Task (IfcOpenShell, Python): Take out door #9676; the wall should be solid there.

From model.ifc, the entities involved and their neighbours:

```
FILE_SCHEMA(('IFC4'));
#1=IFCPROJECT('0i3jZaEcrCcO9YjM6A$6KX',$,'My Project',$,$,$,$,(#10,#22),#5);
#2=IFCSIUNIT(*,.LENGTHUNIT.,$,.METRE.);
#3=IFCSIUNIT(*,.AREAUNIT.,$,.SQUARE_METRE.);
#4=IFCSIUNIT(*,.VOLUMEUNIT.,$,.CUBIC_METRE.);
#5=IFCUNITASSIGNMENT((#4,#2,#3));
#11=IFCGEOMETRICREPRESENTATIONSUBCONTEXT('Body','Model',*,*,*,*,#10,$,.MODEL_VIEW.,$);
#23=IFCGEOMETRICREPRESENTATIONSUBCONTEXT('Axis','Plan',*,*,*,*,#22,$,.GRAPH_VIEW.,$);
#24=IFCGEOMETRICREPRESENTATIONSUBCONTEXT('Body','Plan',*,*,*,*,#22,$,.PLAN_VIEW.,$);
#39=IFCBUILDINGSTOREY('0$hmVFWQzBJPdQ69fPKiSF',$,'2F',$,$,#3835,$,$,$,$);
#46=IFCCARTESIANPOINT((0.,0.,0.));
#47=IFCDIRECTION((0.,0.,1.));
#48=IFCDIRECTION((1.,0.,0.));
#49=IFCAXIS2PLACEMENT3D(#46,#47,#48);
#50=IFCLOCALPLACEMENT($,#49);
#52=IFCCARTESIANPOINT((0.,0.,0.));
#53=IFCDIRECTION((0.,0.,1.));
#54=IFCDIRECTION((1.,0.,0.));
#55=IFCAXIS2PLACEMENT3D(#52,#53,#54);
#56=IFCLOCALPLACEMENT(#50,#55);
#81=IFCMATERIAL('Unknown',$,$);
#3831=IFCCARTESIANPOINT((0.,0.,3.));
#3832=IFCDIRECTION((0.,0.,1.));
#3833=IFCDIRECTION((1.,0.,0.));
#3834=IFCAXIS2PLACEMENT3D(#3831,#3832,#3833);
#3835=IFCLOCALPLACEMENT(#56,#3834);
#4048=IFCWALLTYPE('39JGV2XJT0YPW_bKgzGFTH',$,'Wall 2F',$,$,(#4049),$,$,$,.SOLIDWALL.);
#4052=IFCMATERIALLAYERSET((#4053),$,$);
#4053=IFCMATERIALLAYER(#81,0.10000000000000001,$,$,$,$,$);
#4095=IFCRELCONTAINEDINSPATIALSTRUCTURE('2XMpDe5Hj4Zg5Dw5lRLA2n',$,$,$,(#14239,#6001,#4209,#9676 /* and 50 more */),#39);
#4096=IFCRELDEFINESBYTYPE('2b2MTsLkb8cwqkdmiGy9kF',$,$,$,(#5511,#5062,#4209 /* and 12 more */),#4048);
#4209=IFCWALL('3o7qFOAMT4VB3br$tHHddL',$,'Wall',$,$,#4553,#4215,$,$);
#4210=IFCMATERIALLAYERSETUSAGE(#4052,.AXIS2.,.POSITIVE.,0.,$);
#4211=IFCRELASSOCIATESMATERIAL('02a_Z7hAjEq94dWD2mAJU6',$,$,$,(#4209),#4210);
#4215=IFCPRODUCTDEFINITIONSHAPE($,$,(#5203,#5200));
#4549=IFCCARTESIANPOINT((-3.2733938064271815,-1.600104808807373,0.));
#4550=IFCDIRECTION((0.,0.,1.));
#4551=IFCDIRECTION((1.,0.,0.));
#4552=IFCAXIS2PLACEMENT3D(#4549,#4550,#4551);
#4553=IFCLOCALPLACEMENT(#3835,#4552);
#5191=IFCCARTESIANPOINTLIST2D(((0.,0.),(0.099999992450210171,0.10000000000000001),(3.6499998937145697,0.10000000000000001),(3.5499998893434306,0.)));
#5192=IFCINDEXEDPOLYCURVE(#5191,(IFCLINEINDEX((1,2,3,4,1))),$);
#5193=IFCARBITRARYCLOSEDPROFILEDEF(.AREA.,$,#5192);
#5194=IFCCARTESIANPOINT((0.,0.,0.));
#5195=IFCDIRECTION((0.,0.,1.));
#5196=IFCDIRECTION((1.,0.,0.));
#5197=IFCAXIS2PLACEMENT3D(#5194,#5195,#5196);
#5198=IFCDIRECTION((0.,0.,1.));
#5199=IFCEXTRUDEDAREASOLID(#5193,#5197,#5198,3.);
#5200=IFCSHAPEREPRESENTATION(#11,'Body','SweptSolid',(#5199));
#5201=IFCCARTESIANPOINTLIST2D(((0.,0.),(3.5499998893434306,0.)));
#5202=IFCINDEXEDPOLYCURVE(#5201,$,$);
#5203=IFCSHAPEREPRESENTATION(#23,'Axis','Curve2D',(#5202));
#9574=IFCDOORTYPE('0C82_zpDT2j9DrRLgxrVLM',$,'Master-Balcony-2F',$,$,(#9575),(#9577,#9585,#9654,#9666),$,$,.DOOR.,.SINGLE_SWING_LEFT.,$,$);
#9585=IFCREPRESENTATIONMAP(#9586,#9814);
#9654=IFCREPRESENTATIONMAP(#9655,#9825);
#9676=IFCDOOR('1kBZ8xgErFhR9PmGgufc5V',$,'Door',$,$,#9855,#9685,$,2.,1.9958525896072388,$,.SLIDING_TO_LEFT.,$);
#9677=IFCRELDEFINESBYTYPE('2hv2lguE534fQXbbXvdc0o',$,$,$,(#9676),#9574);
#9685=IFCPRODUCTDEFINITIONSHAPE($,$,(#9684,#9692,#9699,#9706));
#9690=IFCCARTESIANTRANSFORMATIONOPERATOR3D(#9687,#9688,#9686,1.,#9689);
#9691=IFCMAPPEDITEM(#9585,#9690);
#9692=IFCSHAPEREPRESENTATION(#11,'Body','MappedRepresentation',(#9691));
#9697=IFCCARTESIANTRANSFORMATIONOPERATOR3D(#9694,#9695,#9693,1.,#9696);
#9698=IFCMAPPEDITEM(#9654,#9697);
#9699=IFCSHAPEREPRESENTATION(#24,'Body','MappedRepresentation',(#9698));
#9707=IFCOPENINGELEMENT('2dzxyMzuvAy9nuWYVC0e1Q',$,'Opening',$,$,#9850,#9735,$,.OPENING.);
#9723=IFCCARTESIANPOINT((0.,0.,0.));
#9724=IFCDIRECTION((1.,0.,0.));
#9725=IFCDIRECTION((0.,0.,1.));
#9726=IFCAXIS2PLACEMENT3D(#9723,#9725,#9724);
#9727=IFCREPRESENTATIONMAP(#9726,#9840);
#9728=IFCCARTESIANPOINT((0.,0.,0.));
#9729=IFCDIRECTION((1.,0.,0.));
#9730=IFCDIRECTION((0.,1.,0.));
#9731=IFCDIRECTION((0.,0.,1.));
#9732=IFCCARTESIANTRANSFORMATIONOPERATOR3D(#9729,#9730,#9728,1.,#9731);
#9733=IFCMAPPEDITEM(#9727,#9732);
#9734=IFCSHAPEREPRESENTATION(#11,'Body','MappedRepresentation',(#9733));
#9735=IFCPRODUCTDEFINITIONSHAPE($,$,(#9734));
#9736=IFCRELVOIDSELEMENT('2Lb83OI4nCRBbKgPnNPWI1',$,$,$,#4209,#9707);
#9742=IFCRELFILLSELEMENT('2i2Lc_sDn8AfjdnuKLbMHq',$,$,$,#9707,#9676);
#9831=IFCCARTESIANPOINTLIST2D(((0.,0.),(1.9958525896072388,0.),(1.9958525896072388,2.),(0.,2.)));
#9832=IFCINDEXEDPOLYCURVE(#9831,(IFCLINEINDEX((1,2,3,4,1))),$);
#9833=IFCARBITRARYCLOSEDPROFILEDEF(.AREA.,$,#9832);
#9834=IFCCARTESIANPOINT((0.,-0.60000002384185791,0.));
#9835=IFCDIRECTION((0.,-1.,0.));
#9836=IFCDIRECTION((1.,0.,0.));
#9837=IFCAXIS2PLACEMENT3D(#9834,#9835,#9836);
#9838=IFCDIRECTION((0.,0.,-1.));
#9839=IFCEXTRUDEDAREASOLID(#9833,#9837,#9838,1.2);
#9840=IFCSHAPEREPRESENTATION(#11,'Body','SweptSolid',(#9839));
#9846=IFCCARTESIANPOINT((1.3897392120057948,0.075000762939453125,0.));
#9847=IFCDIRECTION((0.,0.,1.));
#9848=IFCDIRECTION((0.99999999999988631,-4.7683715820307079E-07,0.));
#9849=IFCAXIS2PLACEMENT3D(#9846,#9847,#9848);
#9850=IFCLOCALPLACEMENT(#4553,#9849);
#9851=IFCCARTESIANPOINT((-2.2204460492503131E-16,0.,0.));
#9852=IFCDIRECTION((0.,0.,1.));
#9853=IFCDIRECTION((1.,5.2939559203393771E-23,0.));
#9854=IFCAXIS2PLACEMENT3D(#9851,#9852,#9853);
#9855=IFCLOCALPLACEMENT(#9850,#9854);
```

```python
import ifcopenshell
import ifcopenshell.api.feature
import ifcopenshell.api.root
import ifcopenshell.geom
import ifcopenshell.util.shape

model = ifcopenshell.open("model.ifc")
settings = ifcopenshell.geom.settings()


def volume(element):
    """Net volume in cubic metres, openings subtracted."""
    shape = ifcopenshell.geom.create_shape(settings, element)
    return ifcopenshell.util.shape.get_volume(shape.geometry)


door = model.by_guid("1kBZ8xgErFhR9PmGgufc5V")
opening = door.FillsVoids[0].RelatingOpeningElement
wall = opening.VoidsElements[0].RelatingBuildingElement
before = volume(wall)

ifcopenshell.api.root.remove_product(model, product=door)
ifcopenshell.api.feature.remove_feature(model, feature=opening)

after = volume(wall)

print(f"wall volume {before:.3f} -> {after:.3f} m3")

model.write("model-out.ifc")
```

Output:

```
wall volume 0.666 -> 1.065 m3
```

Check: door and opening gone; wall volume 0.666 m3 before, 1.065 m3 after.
